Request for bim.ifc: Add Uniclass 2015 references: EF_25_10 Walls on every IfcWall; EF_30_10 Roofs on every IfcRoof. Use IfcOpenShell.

First a look at what the model holds.

```python
import ifcopenshell

model = ifcopenshell.open("bim.ifc")
print(model.schema)
print("classifications:", [c.Name for c in model.by_type("IfcClassification")])
for ifc_class in ("IfcDoor", "IfcRoof", "IfcStair", "IfcWall", "IfcWindow"):
    print(ifc_class, len(model.by_type(ifc_class)))
```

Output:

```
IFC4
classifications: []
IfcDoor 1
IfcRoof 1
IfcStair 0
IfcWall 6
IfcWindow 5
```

```python
import ifcopenshell
import ifcopenshell.api.classification

model = ifcopenshell.open("bim.ifc")

system = ifcopenshell.api.classification.add_classification(model, classification="Uniclass 2015")

codes = {
    "IfcWall": ("EF_25_10", "Walls"),
    "IfcRoof": ("EF_30_10", "Roofs"),
}
for ifc_class, (code, name) in codes.items():
    products = model.by_type(ifc_class)
    ifcopenshell.api.classification.add_reference(
        model, products=products, classification=system, identification=code, name=name
    )
    print(code, len(products))

model.write("bim_updated.ifc")
```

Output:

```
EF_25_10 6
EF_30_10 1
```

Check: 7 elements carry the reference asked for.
